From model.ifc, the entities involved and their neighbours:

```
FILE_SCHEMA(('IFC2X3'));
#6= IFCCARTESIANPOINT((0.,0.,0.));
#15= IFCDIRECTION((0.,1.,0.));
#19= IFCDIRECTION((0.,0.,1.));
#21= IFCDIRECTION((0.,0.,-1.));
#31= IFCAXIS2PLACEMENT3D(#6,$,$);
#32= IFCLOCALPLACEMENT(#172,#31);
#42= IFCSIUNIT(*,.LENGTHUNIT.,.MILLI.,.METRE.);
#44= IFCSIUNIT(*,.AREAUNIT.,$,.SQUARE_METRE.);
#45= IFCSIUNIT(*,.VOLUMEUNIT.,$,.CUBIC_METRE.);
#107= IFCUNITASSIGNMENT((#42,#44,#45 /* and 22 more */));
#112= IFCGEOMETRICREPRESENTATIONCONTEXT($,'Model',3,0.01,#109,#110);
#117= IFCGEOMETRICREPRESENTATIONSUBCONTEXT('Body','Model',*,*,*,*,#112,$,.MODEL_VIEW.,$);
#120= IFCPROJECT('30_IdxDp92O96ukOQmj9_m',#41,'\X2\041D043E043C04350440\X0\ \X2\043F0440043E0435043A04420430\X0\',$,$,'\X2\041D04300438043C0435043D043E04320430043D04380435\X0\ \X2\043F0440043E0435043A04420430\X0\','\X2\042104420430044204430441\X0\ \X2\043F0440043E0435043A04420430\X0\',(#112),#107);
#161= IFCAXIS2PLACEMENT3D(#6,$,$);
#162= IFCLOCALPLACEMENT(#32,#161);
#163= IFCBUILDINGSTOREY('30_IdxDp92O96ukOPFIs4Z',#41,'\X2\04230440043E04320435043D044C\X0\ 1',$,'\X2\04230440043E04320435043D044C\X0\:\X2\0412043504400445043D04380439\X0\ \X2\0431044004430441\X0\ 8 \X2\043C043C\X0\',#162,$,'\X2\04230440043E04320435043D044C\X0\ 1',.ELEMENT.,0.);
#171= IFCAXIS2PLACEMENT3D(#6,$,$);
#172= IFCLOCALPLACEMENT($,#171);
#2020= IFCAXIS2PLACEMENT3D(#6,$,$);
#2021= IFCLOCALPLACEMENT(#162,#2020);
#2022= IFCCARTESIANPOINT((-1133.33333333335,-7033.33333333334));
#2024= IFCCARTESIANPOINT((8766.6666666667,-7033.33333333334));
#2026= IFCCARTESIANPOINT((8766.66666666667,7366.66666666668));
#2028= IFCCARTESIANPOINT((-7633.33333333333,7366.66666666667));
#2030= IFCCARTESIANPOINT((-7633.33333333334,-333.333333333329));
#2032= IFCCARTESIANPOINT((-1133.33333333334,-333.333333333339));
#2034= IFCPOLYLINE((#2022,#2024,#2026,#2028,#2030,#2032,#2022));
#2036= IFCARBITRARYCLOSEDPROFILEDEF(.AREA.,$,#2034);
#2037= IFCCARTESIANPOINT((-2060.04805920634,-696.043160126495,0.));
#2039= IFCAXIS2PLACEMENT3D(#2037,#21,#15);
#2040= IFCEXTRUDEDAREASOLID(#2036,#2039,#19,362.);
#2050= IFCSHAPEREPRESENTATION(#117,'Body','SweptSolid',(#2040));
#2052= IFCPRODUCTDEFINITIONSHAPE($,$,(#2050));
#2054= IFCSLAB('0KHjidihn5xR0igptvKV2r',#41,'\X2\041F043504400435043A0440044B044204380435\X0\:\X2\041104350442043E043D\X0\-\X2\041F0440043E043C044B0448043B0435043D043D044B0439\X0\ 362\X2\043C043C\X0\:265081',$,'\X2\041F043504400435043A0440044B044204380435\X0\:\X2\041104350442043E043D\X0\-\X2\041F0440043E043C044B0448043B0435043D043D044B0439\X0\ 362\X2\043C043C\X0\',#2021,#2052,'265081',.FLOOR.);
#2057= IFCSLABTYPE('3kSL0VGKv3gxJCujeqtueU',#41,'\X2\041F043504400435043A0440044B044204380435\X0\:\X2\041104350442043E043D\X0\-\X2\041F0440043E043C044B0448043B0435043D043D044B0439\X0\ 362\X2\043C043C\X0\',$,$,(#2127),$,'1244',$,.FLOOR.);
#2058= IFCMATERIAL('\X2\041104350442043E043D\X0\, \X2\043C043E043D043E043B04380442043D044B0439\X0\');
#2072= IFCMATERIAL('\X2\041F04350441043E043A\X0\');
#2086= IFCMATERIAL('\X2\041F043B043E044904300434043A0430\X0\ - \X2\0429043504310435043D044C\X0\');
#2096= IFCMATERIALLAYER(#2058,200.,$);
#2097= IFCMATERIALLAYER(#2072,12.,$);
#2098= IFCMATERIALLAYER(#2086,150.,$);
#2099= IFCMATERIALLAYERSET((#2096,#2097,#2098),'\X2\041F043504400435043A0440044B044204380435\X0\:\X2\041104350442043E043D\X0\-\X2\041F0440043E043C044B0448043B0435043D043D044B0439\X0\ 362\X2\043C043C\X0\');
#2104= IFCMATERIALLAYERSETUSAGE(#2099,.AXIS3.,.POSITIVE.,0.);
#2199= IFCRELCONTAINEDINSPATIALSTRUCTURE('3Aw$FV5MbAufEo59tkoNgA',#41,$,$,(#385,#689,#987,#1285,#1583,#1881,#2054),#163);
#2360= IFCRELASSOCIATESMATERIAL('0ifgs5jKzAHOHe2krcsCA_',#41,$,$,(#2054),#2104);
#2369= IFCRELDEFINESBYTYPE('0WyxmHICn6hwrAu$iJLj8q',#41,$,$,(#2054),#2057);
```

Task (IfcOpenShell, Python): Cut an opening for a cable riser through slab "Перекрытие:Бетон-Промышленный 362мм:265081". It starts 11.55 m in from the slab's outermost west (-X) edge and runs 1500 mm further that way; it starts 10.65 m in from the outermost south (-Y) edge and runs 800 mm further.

```python
import numpy as np
import ifcopenshell
import ifcopenshell.api.feature
import ifcopenshell.api.geometry
import ifcopenshell.api.root
import ifcopenshell.geom
import ifcopenshell.util.placement
import ifcopenshell.util.representation
import ifcopenshell.util.shape
import ifcopenshell.util.unit

model = ifcopenshell.open("model.ifc")
unit_scale = ifcopenshell.util.unit.calculate_unit_scale(model)
settings = ifcopenshell.geom.settings()


def volume(element):
    """Net volume in cubic metres, openings subtracted."""
    shape = ifcopenshell.geom.create_shape(settings, element)
    return ifcopenshell.util.shape.get_volume(shape.geometry)


slab = model.by_id(2054)
before = volume(slab)

# Extent in the slab's own axes, in metres. The edges named are its -X and -Y sides.
slab_shape = ifcopenshell.geom.create_shape(settings, slab)
vertices = ifcopenshell.util.shape.get_vertices(slab_shape.geometry)
x_min, y_min, bottom = vertices.min(axis=0)
top = vertices[:, 2].max()

opening = ifcopenshell.api.root.create_entity(model, ifc_class="IfcOpeningElement", name="Cable riser opening")
context = ifcopenshell.util.representation.get_context(model, "Model", "Body", "MODEL_VIEW")
width, depth = 1.5, 0.8
outline = [(0.0, 0.0), (width, 0.0), (width, depth), (0.0, depth), (0.0, 0.0)]
# Overshoot both faces by 50 mm so the cut is clean.
shape = ifcopenshell.api.geometry.add_slab_representation(
    model, context=context, depth=top - bottom + 0.1, polyline=outline
)
ifcopenshell.api.geometry.assign_representation(model, product=opening, representation=shape)

matrix = ifcopenshell.util.placement.get_local_placement(slab.ObjectPlacement)
matrix[:, 3] = matrix @ np.append(np.array([x_min + 11.55, y_min + 10.65, bottom - 0.05]) / unit_scale, 1.0)
ifcopenshell.api.geometry.edit_object_placement(model, product=opening, matrix=matrix, is_si=False)
ifcopenshell.api.feature.add_feature(model, feature=opening, element=slab)

after = volume(slab)

print(f"slab volume {before:.3f} -> {after:.3f} m3")

model.write("model_edited.ifc")
```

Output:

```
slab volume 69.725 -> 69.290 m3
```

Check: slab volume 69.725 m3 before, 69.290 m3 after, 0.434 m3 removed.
